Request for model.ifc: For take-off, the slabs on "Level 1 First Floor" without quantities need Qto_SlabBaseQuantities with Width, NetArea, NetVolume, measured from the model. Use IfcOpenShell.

First a look at what the model holds.

```python
import ifcopenshell
import ifcopenshell.util.element
import ifcopenshell.util.unit

model = ifcopenshell.open("model.ifc")
print(model.schema)
for unit_type in ("LENGTHUNIT", "AREAUNIT", "VOLUMEUNIT"):
    print(unit_type, ifcopenshell.util.unit.calculate_unit_scale(model, unit_type))
storey = next(s for s in model.by_type("IfcBuildingStorey") if s.Name == "Level 1 First Floor")
slabs = [e for e in ifcopenshell.util.element.get_decomposition(storey) if e.is_a("IfcSlab")]
for e in sorted(slabs, key=lambda e: e.id()):
    print(e.id(), e.is_a(), e.Name, list(ifcopenshell.util.element.get_psets(e, qtos_only=True)), sep=" | ")
```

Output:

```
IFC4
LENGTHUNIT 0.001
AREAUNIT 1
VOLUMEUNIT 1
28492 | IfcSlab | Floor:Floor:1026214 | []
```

```python
import ifcopenshell
import ifcopenshell.api.pset
import ifcopenshell.geom
import ifcopenshell.util.element
import ifcopenshell.util.shape
import ifcopenshell.util.unit

model = ifcopenshell.open("model.ifc")
unit_scale = ifcopenshell.util.unit.calculate_unit_scale(model)
area_scale = ifcopenshell.util.unit.calculate_unit_scale(model, "AREAUNIT")
volume_scale = ifcopenshell.util.unit.calculate_unit_scale(model, "VOLUMEUNIT")
settings = ifcopenshell.geom.settings()

storey = next(s for s in model.by_type("IfcBuildingStorey") if s.Name == "Level 1 First Floor")
slabs = [e for e in ifcopenshell.util.element.get_decomposition(storey) if e.is_a("IfcSlab")]

for e in sorted(slabs, key=lambda e: e.id()):
    if ifcopenshell.util.element.get_psets(e, qtos_only=True, should_inherit=False):
        continue
    # Geometry comes back in metres, in the element's own axes.
    shape = ifcopenshell.geom.create_shape(settings, e)
    values = {
        "Width": ifcopenshell.util.shape.get_z(shape.geometry) / unit_scale,
        "NetArea": ifcopenshell.util.shape.get_footprint_area(shape.geometry) / area_scale,
        "NetVolume": ifcopenshell.util.shape.get_volume(shape.geometry) / volume_scale,
    }
    qto = ifcopenshell.api.pset.add_qto(model, product=e, name="Qto_SlabBaseQuantities")
    ifcopenshell.api.pset.edit_qto(model, qto=qto, properties=values)
    print(e.id(), {k: round(v, 3) for k, v in values.items()})

model.write("model_v2.ifc")
```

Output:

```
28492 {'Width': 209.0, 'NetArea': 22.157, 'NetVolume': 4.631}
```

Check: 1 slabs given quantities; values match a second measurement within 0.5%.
